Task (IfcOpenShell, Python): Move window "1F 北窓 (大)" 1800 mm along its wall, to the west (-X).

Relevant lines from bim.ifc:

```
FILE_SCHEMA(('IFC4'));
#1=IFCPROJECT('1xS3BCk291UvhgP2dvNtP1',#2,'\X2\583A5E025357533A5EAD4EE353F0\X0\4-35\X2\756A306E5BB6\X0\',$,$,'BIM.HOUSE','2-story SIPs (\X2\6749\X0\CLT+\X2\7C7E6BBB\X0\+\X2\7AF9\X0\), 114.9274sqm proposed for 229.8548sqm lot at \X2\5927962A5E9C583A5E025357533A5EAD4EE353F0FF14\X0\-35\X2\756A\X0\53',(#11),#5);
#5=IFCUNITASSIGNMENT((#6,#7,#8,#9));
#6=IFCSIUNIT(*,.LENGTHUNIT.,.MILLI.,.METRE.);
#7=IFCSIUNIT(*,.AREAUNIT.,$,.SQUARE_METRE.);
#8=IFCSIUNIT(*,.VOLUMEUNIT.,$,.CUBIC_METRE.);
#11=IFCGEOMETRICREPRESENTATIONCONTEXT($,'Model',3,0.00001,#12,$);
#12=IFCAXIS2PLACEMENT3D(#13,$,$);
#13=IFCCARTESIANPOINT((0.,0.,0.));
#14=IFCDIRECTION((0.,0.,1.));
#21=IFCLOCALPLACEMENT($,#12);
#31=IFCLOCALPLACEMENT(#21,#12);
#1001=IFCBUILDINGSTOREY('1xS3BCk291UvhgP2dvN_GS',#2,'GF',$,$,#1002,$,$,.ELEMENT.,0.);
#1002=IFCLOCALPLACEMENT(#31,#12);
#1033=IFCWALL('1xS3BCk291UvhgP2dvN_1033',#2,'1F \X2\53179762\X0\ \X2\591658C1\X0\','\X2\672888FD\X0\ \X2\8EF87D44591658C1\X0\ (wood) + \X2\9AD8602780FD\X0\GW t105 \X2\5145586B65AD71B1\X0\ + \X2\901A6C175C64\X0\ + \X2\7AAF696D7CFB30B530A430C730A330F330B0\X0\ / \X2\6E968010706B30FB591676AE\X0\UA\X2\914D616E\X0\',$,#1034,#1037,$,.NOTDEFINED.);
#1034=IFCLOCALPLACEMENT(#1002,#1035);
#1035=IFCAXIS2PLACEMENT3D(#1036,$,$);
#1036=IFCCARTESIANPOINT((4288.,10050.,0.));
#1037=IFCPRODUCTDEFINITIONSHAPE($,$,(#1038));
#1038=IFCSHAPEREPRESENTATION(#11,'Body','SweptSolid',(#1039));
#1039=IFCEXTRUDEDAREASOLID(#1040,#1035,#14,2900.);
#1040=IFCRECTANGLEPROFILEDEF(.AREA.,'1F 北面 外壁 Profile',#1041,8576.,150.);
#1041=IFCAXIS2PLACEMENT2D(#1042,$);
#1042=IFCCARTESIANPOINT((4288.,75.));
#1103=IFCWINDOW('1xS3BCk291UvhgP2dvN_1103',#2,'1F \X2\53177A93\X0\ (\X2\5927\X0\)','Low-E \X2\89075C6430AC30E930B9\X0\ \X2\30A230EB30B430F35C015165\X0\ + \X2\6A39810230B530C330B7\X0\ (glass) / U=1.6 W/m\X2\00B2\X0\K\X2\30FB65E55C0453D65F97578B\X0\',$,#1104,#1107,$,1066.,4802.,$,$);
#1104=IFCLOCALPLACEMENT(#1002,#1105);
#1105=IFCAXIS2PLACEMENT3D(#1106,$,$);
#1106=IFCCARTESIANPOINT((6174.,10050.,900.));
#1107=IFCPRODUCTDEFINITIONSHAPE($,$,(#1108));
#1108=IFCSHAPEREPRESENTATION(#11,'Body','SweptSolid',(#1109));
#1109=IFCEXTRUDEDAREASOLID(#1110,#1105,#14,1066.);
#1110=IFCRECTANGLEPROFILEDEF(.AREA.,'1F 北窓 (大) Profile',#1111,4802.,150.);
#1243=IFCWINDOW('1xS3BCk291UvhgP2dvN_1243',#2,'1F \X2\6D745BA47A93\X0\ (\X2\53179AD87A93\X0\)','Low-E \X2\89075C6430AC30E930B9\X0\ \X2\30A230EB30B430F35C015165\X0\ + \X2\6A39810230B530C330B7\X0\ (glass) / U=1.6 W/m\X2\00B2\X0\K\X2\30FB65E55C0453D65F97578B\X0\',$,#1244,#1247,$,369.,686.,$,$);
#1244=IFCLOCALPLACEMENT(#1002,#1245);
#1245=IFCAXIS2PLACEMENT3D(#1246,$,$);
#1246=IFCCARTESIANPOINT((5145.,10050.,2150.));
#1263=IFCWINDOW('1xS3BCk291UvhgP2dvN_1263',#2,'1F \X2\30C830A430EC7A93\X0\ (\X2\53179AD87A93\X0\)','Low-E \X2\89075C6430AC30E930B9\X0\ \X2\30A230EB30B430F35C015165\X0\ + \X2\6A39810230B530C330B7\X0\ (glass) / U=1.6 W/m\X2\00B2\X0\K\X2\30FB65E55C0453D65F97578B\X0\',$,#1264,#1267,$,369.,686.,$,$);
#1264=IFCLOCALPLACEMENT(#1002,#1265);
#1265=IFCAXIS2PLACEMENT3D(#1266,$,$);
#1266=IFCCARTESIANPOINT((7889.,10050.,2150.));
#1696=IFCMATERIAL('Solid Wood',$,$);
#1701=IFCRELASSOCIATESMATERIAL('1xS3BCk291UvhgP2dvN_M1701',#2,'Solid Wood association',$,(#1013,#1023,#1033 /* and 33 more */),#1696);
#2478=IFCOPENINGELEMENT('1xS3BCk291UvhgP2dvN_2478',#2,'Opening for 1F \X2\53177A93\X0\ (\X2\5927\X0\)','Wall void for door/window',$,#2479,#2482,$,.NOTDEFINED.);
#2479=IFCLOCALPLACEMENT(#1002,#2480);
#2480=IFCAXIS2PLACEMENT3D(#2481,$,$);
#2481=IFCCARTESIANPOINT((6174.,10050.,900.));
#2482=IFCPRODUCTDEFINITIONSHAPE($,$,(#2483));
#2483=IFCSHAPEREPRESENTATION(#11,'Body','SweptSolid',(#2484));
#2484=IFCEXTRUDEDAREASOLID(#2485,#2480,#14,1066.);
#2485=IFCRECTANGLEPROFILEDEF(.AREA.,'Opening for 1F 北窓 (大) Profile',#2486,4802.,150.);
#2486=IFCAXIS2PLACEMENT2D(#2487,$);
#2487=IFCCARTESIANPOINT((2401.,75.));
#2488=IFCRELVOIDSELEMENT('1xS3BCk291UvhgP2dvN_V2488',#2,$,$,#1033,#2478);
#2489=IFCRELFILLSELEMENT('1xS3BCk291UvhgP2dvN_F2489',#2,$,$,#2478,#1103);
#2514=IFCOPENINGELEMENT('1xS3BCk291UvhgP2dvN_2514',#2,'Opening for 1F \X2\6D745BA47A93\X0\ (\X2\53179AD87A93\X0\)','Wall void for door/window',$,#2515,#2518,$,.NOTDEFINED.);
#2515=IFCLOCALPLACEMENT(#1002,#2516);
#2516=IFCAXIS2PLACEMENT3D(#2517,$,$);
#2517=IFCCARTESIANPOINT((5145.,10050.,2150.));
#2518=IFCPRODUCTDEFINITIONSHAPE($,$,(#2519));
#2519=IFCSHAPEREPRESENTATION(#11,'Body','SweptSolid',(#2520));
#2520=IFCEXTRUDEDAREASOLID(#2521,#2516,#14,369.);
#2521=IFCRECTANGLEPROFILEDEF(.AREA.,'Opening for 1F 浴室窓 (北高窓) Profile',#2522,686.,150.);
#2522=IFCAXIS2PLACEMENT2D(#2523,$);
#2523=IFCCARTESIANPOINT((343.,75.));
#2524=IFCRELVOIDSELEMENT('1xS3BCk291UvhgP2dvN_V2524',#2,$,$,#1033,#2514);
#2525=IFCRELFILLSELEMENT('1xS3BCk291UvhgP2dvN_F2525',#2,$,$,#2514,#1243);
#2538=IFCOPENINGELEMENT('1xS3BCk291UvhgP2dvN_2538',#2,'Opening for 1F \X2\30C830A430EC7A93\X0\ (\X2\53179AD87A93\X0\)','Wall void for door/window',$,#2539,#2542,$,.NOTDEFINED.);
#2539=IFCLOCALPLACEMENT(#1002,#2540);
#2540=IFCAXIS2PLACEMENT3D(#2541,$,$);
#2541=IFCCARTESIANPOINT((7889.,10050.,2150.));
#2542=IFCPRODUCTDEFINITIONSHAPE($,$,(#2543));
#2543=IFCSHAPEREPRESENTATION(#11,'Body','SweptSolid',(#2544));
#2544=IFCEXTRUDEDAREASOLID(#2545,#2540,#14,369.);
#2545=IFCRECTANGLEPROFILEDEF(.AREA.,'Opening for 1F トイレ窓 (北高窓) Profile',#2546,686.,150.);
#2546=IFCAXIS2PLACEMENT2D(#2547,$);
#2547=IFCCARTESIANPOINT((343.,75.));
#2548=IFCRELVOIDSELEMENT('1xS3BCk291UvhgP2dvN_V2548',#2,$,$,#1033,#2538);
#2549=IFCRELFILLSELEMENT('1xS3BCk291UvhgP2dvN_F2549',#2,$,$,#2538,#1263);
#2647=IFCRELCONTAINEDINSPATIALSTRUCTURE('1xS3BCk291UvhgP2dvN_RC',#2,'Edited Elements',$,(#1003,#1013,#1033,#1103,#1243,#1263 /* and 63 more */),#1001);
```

```python
import ifcopenshell
import ifcopenshell.api.geometry
import ifcopenshell.util.placement
import ifcopenshell.util.unit

model = ifcopenshell.open("bim.ifc")
unit_scale = ifcopenshell.util.unit.calculate_unit_scale(model)

window = model.by_id(1103)
opening = window.FillsVoids[0].RelatingOpeningElement
wall = opening.VoidsElements[0].RelatingBuildingElement

wall_matrix = ifcopenshell.util.placement.get_local_placement(wall.ObjectPlacement)
shift = wall_matrix[:3, 0] * -1.8 / unit_scale
before = ifcopenshell.util.placement.get_local_placement(window.ObjectPlacement)[:3, 3].copy()

# The window is not placed relative to its opening, so move both.
for product in (opening, window):
    matrix = ifcopenshell.util.placement.get_local_placement(product.ObjectPlacement)
    matrix[:3, 3] += shift
    ifcopenshell.api.geometry.edit_object_placement(model, product=product, matrix=matrix, is_si=False)

after = ifcopenshell.util.placement.get_local_placement(window.ObjectPlacement)[:3, 3]
print("window moved by", (after - before).round(3) + 0.0)

model.write("bim_updated.ifc")
```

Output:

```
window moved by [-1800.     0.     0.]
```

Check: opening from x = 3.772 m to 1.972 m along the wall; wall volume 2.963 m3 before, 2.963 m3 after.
